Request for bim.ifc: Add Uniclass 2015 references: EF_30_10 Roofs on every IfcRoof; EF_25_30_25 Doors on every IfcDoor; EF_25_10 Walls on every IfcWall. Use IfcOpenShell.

First a look at what the model holds.

```python
import ifcopenshell

model = ifcopenshell.open("bim.ifc")
print(model.schema)
print("classifications:", [c.Name for c in model.by_type("IfcClassification")])
for ifc_class in ("IfcDoor", "IfcRoof", "IfcStair", "IfcWall", "IfcWindow"):
    print(ifc_class, len(model.by_type(ifc_class)))
```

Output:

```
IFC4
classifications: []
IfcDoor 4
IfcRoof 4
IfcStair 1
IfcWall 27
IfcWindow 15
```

```python
import ifcopenshell
import ifcopenshell.api.classification

model = ifcopenshell.open("bim.ifc")

system = ifcopenshell.api.classification.add_classification(model, classification="Uniclass 2015")

codes = {
    "IfcRoof": ("EF_30_10", "Roofs"),
    "IfcDoor": ("EF_25_30_25", "Doors"),
    "IfcWall": ("EF_25_10", "Walls"),
}
for ifc_class, (code, name) in codes.items():
    products = model.by_type(ifc_class)
    ifcopenshell.api.classification.add_reference(
        model, products=products, classification=system, identification=code, name=name
    )
    print(code, len(products))

model.write("bim_edited.ifc")
```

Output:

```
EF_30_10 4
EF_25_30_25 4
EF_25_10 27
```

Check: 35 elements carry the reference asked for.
